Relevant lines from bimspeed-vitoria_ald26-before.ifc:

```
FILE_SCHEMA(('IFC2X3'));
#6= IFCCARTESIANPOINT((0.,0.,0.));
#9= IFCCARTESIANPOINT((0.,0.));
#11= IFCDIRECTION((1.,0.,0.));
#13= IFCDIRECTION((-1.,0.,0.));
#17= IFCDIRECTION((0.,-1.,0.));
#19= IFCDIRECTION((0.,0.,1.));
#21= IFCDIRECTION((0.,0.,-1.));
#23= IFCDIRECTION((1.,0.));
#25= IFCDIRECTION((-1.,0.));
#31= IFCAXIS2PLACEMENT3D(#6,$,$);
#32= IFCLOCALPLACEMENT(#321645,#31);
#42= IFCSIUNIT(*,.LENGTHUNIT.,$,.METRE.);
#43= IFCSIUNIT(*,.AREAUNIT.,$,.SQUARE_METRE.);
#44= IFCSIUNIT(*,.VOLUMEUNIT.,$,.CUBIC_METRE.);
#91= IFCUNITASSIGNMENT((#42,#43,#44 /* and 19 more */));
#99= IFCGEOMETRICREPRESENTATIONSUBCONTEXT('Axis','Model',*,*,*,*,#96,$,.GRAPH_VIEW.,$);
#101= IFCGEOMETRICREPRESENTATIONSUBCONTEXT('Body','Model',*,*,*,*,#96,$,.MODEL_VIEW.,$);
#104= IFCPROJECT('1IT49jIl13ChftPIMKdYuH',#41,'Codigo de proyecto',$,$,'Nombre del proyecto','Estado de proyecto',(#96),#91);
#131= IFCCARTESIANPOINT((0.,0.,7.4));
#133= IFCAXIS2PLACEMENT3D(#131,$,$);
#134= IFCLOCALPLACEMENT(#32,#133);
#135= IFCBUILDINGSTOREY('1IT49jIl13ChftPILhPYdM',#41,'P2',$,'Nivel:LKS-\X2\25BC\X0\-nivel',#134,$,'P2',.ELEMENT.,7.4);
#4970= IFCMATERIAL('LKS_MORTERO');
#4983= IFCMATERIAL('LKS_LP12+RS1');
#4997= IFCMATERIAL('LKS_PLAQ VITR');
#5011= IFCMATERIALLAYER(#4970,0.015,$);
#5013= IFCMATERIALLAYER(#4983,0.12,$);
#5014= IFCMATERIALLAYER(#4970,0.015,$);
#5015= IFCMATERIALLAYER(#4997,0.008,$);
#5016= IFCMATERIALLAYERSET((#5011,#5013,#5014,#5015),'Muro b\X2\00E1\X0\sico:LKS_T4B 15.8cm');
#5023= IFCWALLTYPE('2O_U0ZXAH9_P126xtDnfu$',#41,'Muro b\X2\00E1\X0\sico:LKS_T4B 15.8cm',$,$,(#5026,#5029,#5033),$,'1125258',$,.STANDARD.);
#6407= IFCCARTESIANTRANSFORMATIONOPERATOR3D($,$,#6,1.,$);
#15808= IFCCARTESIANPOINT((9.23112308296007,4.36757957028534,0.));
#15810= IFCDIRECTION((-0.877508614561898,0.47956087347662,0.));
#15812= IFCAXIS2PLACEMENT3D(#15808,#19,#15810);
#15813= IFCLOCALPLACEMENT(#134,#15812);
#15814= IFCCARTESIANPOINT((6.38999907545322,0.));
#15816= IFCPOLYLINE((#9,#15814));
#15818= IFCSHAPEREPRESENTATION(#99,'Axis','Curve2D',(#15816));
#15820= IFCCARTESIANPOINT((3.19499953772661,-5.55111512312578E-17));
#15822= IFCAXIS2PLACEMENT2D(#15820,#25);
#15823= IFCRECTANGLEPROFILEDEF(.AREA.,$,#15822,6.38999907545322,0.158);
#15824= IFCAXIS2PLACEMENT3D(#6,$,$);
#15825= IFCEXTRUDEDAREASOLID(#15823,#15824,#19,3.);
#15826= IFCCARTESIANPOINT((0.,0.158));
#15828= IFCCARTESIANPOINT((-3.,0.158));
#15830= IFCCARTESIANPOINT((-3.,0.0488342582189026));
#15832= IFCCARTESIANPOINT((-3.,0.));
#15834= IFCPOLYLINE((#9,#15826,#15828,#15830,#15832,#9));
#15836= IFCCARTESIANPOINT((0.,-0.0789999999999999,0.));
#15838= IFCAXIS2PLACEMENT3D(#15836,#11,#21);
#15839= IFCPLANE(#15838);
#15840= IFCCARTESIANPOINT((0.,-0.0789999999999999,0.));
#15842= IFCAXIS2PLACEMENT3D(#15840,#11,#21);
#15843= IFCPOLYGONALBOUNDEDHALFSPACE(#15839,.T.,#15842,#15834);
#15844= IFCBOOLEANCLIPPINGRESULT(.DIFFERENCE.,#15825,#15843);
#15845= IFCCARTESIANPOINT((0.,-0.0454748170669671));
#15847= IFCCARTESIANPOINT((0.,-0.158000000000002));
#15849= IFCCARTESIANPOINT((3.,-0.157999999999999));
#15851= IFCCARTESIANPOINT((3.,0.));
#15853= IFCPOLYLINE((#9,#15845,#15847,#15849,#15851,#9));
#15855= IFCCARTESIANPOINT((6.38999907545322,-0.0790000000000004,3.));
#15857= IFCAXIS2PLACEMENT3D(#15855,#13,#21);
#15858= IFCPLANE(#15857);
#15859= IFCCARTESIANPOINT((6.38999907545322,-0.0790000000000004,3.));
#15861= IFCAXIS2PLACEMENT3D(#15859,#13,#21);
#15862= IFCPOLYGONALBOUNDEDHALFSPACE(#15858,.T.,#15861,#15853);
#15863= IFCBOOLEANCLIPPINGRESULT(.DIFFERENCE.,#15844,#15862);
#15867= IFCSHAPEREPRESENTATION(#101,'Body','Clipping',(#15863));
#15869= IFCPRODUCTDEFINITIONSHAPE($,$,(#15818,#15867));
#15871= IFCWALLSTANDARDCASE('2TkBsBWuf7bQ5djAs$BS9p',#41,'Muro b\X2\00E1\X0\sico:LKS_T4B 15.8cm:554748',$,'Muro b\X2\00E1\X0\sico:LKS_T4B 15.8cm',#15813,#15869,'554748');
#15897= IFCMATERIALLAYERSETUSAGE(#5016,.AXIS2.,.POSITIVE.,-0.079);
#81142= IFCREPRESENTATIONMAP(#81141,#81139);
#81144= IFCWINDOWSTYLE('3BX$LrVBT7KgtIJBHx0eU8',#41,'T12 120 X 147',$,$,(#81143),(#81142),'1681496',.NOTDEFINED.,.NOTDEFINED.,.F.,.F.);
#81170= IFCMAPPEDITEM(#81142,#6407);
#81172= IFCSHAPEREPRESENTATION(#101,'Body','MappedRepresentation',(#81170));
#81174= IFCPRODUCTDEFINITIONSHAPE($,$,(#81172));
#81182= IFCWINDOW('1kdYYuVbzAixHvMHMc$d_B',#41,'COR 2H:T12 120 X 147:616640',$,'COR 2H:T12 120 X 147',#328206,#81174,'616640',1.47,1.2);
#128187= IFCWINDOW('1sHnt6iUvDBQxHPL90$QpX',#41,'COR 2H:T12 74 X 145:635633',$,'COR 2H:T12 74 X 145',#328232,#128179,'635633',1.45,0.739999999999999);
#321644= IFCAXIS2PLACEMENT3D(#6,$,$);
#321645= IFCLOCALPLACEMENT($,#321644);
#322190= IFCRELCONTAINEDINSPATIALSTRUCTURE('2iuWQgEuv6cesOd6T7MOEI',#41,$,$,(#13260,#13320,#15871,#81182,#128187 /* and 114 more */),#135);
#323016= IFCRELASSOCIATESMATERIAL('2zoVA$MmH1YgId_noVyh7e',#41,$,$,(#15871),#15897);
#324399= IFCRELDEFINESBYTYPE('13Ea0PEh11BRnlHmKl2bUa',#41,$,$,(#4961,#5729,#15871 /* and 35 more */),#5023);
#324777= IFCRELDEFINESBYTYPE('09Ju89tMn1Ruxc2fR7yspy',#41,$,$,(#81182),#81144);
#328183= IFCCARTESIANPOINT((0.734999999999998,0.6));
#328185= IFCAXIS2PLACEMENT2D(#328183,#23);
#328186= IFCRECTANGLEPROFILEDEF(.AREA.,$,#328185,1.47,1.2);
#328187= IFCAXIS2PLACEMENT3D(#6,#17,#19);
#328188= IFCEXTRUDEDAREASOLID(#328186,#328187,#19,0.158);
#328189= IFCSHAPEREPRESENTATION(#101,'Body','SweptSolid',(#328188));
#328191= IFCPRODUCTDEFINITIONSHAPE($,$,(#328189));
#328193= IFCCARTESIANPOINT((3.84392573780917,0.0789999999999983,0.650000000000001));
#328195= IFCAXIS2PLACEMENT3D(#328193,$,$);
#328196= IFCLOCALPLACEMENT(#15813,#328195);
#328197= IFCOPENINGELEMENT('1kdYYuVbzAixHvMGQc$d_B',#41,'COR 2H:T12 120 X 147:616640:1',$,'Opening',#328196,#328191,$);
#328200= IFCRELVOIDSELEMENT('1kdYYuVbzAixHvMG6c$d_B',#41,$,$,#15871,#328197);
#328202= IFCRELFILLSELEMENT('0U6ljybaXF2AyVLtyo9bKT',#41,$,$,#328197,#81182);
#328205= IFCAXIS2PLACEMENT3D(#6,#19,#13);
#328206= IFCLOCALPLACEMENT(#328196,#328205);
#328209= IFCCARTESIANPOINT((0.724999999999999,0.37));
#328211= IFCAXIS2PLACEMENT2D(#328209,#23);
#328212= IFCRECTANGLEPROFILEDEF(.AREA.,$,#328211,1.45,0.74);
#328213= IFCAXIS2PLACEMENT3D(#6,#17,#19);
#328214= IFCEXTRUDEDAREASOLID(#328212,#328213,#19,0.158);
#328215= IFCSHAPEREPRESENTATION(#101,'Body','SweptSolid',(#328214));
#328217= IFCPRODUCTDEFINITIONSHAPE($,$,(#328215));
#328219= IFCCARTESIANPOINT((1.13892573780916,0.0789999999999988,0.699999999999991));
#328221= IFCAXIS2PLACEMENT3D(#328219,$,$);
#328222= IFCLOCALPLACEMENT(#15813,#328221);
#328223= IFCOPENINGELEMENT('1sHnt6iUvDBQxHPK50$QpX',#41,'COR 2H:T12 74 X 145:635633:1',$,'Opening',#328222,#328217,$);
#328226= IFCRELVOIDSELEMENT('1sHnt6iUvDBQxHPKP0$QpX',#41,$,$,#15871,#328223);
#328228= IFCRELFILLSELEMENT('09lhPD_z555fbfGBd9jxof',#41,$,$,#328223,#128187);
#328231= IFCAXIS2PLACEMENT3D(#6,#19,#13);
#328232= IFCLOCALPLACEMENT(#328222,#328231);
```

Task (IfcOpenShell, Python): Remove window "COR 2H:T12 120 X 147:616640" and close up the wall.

```python
import ifcopenshell
import ifcopenshell.api.feature
import ifcopenshell.api.root
import ifcopenshell.geom
import ifcopenshell.util.shape

model = ifcopenshell.open("bimspeed-vitoria_ald26-before.ifc")
settings = ifcopenshell.geom.settings()


def volume(element):
    """Net volume in cubic metres, openings subtracted."""
    shape = ifcopenshell.geom.create_shape(settings, element)
    return ifcopenshell.util.shape.get_volume(shape.geometry)


window = model.by_guid("1kdYYuVbzAixHvMHMc$d_B")
opening = window.FillsVoids[0].RelatingOpeningElement
wall = opening.VoidsElements[0].RelatingBuildingElement
before = volume(wall)

ifcopenshell.api.root.remove_product(model, product=window)
ifcopenshell.api.feature.remove_feature(model, feature=opening)

after = volume(wall)

print(f"wall volume {before:.3f} -> {after:.3f} m3")

model.write("bimspeed-vitoria_ald26-before_v2.ifc")
```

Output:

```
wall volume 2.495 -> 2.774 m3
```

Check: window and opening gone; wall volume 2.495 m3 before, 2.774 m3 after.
